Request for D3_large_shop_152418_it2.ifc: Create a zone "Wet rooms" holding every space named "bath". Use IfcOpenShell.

First a look at what the model holds.

```python
import ifcopenshell

model = ifcopenshell.open("D3_large_shop_152418_it2.ifc")
print(model.schema)
seen = {}
for space in model.by_type("IfcSpace"):
    seen[space.LongName] = seen.get(space.LongName, 0) + 1
for name, count in sorted(seen.items(), key=str):
    print(count, "x", name)
print("zones:", [z.Name for z in model.by_type("IfcZone")][:20])
```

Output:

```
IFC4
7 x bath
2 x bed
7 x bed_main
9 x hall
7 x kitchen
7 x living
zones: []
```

```python
import ifcopenshell
import ifcopenshell.api.group
import ifcopenshell.api.root

model = ifcopenshell.open("D3_large_shop_152418_it2.ifc")

names = {"bath"}
spaces = [s for s in model.by_type("IfcSpace") if s.LongName in names]

zone = ifcopenshell.api.root.create_entity(model, ifc_class="IfcZone", name="Wet rooms")
ifcopenshell.api.group.assign_group(model, products=spaces, group=zone)
print(len(spaces), "spaces in", zone.Name)

model.write("D3_large_shop_152418_it2_edited.ifc")
```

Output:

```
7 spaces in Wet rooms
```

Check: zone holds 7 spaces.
